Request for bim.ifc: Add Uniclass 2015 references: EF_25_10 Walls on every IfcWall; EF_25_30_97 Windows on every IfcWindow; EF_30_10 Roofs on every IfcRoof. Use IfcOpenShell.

First a look at what the model holds.

```python
import ifcopenshell

model = ifcopenshell.open("bim.ifc")
print(model.schema)
print("classifications:", [c.Name for c in model.by_type("IfcClassification")])
for ifc_class in ("IfcDoor", "IfcRoof", "IfcStair", "IfcWall", "IfcWindow"):
    print(ifc_class, len(model.by_type(ifc_class)))
```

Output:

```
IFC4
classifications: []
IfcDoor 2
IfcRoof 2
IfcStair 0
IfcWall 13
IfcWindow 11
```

```python
import ifcopenshell
import ifcopenshell.api.classification

model = ifcopenshell.open("bim.ifc")

system = ifcopenshell.api.classification.add_classification(model, classification="Uniclass 2015")

codes = {
    "IfcWall": ("EF_25_10", "Walls"),
    "IfcWindow": ("EF_25_30_97", "Windows"),
    "IfcRoof": ("EF_30_10", "Roofs"),
}
for ifc_class, (code, name) in codes.items():
    products = model.by_type(ifc_class)
    ifcopenshell.api.classification.add_reference(
        model, products=products, classification=system, identification=code, name=name
    )
    print(code, len(products))

model.write("bim-out.ifc")
```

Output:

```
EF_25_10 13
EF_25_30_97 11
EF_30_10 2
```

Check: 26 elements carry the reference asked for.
